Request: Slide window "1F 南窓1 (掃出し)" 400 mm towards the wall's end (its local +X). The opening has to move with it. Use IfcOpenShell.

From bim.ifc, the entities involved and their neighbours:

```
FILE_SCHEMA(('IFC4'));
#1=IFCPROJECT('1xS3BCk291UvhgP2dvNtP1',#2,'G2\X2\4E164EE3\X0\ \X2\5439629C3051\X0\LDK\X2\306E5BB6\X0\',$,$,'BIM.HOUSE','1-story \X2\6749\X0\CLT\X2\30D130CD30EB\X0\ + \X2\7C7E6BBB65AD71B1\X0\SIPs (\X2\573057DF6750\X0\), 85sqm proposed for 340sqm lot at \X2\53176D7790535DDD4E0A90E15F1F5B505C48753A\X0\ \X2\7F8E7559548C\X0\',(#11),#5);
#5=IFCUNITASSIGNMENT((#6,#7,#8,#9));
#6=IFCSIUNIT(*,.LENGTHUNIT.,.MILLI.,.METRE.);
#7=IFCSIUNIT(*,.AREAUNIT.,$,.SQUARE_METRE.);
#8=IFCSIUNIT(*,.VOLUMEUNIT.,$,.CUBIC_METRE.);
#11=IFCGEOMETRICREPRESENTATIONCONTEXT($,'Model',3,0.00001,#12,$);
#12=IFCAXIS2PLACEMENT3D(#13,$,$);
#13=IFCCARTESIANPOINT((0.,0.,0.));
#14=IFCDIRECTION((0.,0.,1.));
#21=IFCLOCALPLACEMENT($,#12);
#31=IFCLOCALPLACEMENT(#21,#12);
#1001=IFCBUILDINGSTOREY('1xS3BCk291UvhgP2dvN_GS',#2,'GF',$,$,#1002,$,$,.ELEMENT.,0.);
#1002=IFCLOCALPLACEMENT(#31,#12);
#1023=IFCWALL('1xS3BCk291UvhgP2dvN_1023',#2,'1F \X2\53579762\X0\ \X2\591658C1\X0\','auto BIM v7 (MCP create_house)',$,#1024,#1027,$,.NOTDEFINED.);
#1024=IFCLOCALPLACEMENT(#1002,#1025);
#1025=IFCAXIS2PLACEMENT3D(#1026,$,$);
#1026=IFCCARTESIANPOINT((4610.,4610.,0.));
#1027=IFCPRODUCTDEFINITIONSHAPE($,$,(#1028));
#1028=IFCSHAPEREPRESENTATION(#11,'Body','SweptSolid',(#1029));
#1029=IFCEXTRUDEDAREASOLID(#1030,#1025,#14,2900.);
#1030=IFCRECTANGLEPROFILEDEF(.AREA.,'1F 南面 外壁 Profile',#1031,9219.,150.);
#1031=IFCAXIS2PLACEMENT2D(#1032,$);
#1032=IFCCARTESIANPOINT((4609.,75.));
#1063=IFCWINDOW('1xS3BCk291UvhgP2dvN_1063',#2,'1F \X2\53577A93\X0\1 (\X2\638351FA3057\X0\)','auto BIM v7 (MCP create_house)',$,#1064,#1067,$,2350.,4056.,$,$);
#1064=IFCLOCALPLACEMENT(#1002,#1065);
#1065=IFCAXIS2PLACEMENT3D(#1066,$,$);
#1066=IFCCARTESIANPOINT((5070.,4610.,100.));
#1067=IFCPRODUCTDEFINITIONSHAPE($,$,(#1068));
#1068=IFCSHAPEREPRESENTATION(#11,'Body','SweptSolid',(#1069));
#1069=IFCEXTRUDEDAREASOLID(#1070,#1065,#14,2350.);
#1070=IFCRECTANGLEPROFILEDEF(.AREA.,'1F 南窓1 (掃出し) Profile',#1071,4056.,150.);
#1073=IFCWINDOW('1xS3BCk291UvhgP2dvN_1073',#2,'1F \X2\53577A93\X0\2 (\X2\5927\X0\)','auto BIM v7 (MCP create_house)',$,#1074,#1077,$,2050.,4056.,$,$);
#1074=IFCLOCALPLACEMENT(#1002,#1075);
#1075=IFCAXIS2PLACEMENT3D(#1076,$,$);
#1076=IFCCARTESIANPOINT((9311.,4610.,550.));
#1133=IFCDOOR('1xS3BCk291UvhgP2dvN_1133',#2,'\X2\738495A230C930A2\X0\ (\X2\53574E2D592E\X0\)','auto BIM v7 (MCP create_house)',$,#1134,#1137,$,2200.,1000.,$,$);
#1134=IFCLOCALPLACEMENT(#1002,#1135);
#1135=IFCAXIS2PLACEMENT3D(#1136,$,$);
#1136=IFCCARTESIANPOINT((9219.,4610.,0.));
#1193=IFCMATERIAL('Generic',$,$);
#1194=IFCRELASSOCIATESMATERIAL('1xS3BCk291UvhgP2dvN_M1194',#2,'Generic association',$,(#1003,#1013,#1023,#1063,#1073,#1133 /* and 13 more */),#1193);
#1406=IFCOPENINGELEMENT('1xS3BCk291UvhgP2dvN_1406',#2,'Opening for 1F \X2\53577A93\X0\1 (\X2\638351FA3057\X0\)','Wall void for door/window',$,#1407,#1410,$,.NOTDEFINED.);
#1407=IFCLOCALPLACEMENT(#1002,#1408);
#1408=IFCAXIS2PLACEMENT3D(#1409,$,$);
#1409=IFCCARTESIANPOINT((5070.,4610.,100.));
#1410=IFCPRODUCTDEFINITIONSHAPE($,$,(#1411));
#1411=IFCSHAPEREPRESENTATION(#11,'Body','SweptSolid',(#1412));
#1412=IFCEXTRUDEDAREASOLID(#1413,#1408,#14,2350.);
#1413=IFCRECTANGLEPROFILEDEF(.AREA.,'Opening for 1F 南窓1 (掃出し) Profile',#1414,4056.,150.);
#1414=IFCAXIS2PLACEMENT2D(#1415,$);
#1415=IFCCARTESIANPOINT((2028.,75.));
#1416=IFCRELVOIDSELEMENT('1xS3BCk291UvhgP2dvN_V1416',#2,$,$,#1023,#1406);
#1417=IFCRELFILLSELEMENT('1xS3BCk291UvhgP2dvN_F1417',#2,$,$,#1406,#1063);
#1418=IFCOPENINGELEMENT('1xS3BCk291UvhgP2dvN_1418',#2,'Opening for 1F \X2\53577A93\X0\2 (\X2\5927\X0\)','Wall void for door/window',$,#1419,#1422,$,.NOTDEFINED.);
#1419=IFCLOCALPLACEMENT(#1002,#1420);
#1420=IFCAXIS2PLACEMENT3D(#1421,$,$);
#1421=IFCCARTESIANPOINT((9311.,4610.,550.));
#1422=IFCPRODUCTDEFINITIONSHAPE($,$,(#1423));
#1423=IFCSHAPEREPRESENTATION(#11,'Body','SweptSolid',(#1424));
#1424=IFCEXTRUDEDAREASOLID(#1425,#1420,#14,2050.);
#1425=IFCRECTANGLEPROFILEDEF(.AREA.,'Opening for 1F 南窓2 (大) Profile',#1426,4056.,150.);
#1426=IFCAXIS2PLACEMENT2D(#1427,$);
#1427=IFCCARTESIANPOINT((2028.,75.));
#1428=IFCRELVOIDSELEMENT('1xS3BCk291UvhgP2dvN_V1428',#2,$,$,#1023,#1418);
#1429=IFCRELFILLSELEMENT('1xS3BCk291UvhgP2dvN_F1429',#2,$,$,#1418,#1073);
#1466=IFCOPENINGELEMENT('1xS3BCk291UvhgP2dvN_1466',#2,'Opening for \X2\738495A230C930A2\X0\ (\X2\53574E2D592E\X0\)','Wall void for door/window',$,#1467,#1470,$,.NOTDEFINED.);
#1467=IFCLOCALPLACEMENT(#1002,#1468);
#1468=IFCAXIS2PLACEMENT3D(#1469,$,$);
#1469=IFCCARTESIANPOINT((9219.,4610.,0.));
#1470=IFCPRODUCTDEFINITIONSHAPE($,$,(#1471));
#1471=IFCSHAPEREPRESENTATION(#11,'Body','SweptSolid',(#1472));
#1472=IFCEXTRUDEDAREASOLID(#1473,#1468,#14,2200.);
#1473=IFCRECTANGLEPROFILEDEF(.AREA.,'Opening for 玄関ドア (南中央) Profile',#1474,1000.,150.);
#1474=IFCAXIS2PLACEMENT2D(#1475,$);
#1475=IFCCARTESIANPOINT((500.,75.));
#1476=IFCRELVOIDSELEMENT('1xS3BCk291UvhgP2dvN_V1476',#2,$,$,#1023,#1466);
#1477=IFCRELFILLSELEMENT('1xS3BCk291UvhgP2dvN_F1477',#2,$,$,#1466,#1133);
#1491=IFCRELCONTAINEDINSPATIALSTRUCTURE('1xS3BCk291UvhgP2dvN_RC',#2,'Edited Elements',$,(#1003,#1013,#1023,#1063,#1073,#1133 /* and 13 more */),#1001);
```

```python
import ifcopenshell
import ifcopenshell.api.geometry
import ifcopenshell.util.placement
import ifcopenshell.util.unit

model = ifcopenshell.open("bim.ifc")
unit_scale = ifcopenshell.util.unit.calculate_unit_scale(model)

window = model.by_guid("1xS3BCk291UvhgP2dvN_1063")
opening = window.FillsVoids[0].RelatingOpeningElement
wall = opening.VoidsElements[0].RelatingBuildingElement

wall_matrix = ifcopenshell.util.placement.get_local_placement(wall.ObjectPlacement)
shift = wall_matrix[:3, 0] * 0.4 / unit_scale
before = ifcopenshell.util.placement.get_local_placement(window.ObjectPlacement)[:3, 3].copy()

# The window is not placed relative to its opening, so move both.
for product in (opening, window):
    matrix = ifcopenshell.util.placement.get_local_placement(product.ObjectPlacement)
    matrix[:3, 3] += shift
    ifcopenshell.api.geometry.edit_object_placement(model, product=product, matrix=matrix, is_si=False)

after = ifcopenshell.util.placement.get_local_placement(window.ObjectPlacement)[:3, 3]
print("window moved by", (after - before).round(3) + 0.0)

model.write("bim-out.ifc")
```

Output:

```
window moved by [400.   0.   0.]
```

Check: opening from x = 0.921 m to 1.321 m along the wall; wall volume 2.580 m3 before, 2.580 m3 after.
